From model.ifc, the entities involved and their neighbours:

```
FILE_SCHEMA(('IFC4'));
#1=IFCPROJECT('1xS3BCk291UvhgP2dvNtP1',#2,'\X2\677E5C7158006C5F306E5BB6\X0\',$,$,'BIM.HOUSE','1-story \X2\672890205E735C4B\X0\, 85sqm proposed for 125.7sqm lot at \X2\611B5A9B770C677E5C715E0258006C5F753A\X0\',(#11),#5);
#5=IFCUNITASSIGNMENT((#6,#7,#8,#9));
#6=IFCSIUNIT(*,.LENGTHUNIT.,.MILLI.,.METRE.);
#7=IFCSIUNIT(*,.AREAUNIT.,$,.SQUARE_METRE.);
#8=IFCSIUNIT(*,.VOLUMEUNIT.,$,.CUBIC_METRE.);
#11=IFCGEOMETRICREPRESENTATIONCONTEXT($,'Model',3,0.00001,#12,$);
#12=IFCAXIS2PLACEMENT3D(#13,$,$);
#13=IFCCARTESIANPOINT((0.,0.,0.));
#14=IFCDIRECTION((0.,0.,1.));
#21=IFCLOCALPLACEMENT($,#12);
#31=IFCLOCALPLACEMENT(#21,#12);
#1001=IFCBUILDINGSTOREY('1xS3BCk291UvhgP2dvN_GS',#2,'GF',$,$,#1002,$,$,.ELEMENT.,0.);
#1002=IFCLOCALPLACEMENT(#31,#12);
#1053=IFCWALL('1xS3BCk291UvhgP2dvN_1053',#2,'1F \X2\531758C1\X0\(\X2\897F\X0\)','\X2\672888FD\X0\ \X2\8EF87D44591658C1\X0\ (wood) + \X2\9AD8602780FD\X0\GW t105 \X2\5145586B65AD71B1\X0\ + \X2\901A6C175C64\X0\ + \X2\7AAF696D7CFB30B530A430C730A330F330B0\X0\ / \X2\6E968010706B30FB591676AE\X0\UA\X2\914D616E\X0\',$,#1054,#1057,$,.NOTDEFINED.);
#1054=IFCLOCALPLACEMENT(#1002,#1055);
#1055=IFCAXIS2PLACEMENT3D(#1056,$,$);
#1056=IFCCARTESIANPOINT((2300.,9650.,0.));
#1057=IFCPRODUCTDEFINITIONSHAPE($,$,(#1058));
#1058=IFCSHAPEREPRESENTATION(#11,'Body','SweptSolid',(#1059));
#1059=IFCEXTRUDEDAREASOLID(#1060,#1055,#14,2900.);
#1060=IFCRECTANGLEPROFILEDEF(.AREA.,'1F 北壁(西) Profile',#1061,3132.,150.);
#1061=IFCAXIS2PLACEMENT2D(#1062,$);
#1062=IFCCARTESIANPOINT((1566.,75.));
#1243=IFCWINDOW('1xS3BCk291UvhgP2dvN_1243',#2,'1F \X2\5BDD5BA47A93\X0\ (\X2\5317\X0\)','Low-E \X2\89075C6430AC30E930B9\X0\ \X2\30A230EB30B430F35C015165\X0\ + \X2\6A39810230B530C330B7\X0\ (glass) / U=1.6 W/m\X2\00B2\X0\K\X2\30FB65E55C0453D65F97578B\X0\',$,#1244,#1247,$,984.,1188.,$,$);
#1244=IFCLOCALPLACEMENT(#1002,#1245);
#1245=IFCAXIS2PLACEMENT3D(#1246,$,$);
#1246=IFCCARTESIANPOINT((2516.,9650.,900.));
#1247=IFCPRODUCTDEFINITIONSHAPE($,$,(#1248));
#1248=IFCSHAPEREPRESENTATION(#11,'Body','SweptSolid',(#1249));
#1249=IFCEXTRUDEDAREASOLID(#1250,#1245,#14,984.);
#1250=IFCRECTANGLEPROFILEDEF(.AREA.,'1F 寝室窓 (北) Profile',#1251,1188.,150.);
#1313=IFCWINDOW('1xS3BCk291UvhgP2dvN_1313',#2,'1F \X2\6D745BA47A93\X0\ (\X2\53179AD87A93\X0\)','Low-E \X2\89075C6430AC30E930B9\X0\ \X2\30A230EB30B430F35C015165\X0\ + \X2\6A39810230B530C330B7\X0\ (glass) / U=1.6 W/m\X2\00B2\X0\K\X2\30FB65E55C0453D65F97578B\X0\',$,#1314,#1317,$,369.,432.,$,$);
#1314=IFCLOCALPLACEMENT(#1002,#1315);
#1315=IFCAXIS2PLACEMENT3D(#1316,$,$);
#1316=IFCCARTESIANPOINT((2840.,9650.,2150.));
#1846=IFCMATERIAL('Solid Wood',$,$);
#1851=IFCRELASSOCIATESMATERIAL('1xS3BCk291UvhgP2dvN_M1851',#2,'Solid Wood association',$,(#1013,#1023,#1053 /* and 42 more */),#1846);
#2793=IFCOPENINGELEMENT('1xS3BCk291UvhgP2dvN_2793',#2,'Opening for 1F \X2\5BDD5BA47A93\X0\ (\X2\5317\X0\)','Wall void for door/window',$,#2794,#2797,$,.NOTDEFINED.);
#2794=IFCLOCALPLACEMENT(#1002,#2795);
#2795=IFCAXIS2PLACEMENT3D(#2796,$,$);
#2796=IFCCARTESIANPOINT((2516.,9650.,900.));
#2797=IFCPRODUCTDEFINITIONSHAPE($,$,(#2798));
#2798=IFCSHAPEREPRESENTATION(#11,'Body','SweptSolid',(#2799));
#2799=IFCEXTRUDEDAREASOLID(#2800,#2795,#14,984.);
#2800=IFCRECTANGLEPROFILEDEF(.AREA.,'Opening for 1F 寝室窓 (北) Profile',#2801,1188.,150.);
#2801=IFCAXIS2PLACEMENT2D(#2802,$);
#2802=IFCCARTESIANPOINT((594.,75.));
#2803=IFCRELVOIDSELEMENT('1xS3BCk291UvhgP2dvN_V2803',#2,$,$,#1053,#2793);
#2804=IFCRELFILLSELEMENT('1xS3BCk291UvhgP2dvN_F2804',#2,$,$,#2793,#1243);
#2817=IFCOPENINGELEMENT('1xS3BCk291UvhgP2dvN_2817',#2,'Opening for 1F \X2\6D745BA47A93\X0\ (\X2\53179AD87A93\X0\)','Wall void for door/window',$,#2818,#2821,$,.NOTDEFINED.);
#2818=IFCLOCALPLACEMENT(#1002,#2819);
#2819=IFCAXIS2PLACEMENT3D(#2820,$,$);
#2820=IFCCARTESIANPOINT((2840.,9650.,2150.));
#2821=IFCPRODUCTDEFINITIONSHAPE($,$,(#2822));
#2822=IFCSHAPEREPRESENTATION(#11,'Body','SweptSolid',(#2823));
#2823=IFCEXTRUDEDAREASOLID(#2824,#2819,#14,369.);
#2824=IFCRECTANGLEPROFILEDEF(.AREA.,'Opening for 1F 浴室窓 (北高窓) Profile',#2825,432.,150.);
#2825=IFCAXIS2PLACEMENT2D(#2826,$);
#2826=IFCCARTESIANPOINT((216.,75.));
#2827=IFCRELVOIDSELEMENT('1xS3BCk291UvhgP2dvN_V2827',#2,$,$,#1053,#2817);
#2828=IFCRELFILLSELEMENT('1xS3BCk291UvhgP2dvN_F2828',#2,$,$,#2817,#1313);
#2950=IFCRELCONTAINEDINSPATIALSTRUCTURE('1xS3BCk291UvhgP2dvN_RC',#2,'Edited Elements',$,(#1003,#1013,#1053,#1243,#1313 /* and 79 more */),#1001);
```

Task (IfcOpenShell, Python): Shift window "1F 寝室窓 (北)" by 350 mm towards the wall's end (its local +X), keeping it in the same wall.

```python
import ifcopenshell
import ifcopenshell.api.geometry
import ifcopenshell.util.placement
import ifcopenshell.util.unit

model = ifcopenshell.open("model.ifc")
unit_scale = ifcopenshell.util.unit.calculate_unit_scale(model)

window = model.by_guid("1xS3BCk291UvhgP2dvN_1243")
opening = window.FillsVoids[0].RelatingOpeningElement
wall = opening.VoidsElements[0].RelatingBuildingElement

wall_matrix = ifcopenshell.util.placement.get_local_placement(wall.ObjectPlacement)
shift = wall_matrix[:3, 0] * 0.35 / unit_scale
before = ifcopenshell.util.placement.get_local_placement(window.ObjectPlacement)[:3, 3].copy()

# The window is not placed relative to its opening, so move both.
for product in (opening, window):
    matrix = ifcopenshell.util.placement.get_local_placement(product.ObjectPlacement)
    matrix[:3, 3] += shift
    ifcopenshell.api.geometry.edit_object_placement(model, product=product, matrix=matrix, is_si=False)

after = ifcopenshell.util.placement.get_local_placement(window.ObjectPlacement)[:3, 3]
print("window moved by", (after - before).round(3) + 0.0)

model.write("model_v2.ifc")
```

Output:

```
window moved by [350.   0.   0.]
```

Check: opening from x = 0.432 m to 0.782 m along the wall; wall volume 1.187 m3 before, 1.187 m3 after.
